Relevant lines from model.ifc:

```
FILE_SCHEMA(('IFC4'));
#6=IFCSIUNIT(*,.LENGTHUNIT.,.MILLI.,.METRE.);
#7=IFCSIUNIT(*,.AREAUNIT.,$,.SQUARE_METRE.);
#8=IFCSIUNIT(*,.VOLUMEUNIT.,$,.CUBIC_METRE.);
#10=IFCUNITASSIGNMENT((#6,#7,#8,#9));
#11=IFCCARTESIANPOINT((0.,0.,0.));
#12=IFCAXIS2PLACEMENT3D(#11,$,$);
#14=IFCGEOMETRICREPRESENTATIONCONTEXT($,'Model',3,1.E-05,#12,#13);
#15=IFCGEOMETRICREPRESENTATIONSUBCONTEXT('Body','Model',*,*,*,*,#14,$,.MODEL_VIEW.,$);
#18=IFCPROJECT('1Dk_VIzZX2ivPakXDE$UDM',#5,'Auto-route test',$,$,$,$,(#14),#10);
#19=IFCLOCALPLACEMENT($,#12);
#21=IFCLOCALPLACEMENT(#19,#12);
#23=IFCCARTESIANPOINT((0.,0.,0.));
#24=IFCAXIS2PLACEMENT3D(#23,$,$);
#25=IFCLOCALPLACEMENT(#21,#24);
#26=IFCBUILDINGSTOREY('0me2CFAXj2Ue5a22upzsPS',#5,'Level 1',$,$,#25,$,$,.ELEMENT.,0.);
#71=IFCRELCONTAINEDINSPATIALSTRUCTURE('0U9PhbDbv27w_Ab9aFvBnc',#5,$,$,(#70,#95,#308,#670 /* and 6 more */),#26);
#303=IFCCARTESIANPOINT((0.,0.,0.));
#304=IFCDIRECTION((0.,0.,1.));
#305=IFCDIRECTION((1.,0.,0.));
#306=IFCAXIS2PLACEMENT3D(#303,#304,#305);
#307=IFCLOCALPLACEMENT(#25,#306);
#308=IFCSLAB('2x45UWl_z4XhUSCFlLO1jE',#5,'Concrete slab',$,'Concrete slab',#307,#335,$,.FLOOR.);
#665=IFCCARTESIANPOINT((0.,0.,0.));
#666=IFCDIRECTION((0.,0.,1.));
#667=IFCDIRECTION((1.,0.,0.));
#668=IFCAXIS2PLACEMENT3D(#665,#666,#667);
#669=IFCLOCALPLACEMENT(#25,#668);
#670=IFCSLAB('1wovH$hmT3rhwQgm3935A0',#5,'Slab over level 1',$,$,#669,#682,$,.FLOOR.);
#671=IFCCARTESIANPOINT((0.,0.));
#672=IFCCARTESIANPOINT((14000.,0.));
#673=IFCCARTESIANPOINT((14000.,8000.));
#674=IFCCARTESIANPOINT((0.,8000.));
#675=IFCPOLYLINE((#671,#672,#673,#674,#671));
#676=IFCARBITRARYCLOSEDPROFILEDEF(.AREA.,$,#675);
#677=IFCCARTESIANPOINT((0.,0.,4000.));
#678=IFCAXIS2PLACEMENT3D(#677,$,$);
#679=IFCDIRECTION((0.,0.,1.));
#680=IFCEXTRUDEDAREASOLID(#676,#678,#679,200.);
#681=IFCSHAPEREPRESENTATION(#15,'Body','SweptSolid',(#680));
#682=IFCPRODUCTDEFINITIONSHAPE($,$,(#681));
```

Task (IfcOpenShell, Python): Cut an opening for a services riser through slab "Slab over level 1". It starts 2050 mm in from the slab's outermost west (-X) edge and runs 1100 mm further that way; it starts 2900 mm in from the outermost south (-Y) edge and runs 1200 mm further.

```python
import numpy as np
import ifcopenshell
import ifcopenshell.api.feature
import ifcopenshell.api.geometry
import ifcopenshell.api.root
import ifcopenshell.geom
import ifcopenshell.util.placement
import ifcopenshell.util.representation
import ifcopenshell.util.shape
import ifcopenshell.util.unit

model = ifcopenshell.open("model.ifc")
unit_scale = ifcopenshell.util.unit.calculate_unit_scale(model)
settings = ifcopenshell.geom.settings()


def volume(element):
    """Net volume in cubic metres, openings subtracted."""
    shape = ifcopenshell.geom.create_shape(settings, element)
    return ifcopenshell.util.shape.get_volume(shape.geometry)


slab = model.by_id(670)
before = volume(slab)

# Extent in the slab's own axes, in metres. The edges named are its -X and -Y sides.
slab_shape = ifcopenshell.geom.create_shape(settings, slab)
vertices = ifcopenshell.util.shape.get_vertices(slab_shape.geometry)
x_min, y_min, bottom = vertices.min(axis=0)
top = vertices[:, 2].max()

opening = ifcopenshell.api.root.create_entity(model, ifc_class="IfcOpeningElement", name="Services riser opening", predefined_type="OPENING")
context = ifcopenshell.util.representation.get_context(model, "Model", "Body", "MODEL_VIEW")
width, depth = 1.1, 1.2
outline = [(0.0, 0.0), (width, 0.0), (width, depth), (0.0, depth), (0.0, 0.0)]
# Overshoot both faces by 50 mm so the cut is clean.
shape = ifcopenshell.api.geometry.add_slab_representation(
    model, context=context, depth=top - bottom + 0.1, polyline=outline
)
ifcopenshell.api.geometry.assign_representation(model, product=opening, representation=shape)

matrix = ifcopenshell.util.placement.get_local_placement(slab.ObjectPlacement)
matrix[:, 3] = matrix @ np.append(np.array([x_min + 2.05, y_min + 2.9, bottom - 0.05]) / unit_scale, 1.0)
ifcopenshell.api.geometry.edit_object_placement(model, product=opening, matrix=matrix, is_si=False)
ifcopenshell.api.feature.add_feature(model, feature=opening, element=slab)

after = volume(slab)

print(f"slab volume {before:.3f} -> {after:.3f} m3")

model.write("model_v2.ifc")
```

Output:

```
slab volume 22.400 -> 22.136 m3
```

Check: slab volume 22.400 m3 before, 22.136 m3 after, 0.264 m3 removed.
